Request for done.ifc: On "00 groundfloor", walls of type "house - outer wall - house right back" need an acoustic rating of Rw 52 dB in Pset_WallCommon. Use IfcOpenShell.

First a look at what the model holds.

```python
import ifcopenshell
import ifcopenshell.util.element

model = ifcopenshell.open("done.ifc")
print(model.schema)
storey = next(s for s in model.by_type("IfcBuildingStorey") if s.Name == "00 groundfloor")
walls = [e for e in ifcopenshell.util.element.get_decomposition(storey) if e.is_a("IfcWall")]
seen = {}
for e in walls:
    element_type = ifcopenshell.util.element.get_type(e)
    key = (element_type.Name if element_type != e and element_type else None, ifcopenshell.util.element.get_pset(e, "Pset_WallCommon", "AcousticRating"))
    seen[key] = seen.get(key, 0) + 1
for (name, value), count in sorted(seen.items(), key=str):
    print(count, "x", name, "|", value)
```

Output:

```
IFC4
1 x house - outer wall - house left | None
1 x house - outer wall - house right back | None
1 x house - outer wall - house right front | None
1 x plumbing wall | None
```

```python
import ifcopenshell
import ifcopenshell.api.pset
import ifcopenshell.util.element

model = ifcopenshell.open("done.ifc")

storey = next(s for s in model.by_type("IfcBuildingStorey") if s.Name == "00 groundfloor")
walls = [e for e in ifcopenshell.util.element.get_decomposition(storey) if e.is_a("IfcWall")]

count = 0
for e in walls:
    element_type = ifcopenshell.util.element.get_type(e)
    if element_type in (None, e) or element_type.Name != "house - outer wall - house right back":
        continue
    # add_pset returns the element's existing set when there is one.
    pset = ifcopenshell.api.pset.add_pset(model, product=e, name="Pset_WallCommon")
    ifcopenshell.api.pset.edit_pset(model, pset=pset, properties={"AcousticRating": "Rw 52 dB"})
    count += 1

print(count, "walls updated")

model.write("done_rev.ifc")
```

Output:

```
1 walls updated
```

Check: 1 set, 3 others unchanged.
